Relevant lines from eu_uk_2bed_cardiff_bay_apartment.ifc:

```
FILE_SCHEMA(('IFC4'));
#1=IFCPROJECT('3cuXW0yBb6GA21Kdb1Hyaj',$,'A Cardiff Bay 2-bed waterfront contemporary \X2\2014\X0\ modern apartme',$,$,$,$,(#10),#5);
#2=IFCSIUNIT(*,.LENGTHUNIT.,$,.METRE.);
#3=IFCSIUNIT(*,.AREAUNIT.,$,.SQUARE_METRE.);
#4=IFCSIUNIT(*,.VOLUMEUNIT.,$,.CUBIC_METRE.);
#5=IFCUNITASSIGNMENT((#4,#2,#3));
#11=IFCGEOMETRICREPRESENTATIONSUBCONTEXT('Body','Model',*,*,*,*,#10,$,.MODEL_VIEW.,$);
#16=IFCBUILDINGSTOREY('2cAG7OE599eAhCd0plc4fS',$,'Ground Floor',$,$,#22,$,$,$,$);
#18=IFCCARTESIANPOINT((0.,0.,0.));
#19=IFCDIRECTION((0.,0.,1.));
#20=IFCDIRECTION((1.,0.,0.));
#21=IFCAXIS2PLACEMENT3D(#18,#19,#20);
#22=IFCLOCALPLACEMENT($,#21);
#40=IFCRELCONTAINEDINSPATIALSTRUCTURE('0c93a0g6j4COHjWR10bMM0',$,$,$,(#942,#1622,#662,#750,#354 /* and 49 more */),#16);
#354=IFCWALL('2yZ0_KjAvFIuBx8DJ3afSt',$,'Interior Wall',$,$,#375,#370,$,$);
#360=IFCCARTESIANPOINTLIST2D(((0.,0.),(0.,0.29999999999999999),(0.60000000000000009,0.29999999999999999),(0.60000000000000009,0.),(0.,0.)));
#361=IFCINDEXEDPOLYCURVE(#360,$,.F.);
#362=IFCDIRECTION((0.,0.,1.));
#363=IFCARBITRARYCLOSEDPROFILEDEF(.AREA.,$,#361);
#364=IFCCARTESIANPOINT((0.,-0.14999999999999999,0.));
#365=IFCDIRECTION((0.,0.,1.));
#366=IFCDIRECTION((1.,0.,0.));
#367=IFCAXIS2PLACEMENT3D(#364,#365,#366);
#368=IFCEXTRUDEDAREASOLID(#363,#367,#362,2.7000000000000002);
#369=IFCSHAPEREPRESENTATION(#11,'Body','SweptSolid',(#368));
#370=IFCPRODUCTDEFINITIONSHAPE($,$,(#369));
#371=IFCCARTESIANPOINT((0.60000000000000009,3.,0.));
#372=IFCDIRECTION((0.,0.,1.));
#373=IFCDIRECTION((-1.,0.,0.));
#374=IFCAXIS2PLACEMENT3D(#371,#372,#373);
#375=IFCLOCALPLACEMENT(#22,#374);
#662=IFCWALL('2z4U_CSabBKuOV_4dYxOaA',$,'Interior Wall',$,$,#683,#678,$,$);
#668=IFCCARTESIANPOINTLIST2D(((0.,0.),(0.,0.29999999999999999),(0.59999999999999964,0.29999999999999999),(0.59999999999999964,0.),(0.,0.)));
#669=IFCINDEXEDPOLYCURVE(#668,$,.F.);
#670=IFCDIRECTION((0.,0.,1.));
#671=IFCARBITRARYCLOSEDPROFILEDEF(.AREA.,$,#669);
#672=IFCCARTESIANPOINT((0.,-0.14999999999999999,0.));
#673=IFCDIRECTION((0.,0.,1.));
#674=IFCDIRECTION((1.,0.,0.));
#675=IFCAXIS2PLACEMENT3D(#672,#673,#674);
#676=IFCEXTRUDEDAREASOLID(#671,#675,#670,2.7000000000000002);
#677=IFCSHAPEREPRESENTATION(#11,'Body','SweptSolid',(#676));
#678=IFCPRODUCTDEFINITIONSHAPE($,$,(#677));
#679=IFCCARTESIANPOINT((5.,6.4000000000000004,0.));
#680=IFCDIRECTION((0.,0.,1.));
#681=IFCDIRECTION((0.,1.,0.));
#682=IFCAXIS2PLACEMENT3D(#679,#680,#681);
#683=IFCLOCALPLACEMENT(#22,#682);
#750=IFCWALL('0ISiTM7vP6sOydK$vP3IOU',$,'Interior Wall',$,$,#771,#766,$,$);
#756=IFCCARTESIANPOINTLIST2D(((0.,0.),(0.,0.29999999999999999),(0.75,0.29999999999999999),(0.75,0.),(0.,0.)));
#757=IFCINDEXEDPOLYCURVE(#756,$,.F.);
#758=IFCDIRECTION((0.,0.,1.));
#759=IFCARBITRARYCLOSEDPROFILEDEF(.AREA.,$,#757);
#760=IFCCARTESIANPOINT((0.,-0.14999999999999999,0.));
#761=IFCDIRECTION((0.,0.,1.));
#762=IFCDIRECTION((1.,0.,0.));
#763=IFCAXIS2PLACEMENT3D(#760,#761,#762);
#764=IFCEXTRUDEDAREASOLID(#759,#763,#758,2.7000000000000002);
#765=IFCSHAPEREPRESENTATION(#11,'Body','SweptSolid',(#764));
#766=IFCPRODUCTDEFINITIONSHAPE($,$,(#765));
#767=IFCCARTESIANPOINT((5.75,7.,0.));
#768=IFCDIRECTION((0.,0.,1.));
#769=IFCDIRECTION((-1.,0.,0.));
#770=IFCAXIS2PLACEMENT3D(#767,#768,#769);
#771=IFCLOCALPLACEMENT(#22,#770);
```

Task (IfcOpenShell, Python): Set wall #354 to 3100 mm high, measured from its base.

```python
import ifcopenshell
import ifcopenshell.geom
import ifcopenshell.util.representation
import ifcopenshell.util.shape

model = ifcopenshell.open("eu_uk_2bed_cardiff_bay_apartment.ifc")
settings = ifcopenshell.geom.settings()


def volume(element):
    """Net volume in cubic metres, openings subtracted."""
    shape = ifcopenshell.geom.create_shape(settings, element)
    return ifcopenshell.util.shape.get_volume(shape.geometry)


wall = model.by_guid("2yZ0_KjAvFIuBx8DJ3afSt")
before = volume(wall)

body = ifcopenshell.util.representation.get_representation(wall, "Model", "Body")
solid = body.Items[0]
old_height = solid.Depth
solid.Depth = 3.1
after = volume(wall)

print(f"height {old_height:g} -> {solid.Depth:g}, volume {before:.3f} -> {after:.3f} m3")

model.write("eu_uk_2bed_cardiff_bay_apartment_edited.ifc")
```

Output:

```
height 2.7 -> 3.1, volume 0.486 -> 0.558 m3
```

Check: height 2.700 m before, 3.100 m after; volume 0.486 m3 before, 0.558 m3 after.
